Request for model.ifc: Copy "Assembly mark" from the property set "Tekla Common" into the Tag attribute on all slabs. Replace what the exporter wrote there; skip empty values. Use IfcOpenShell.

First a look at what the model holds.

```python
import ifcopenshell
import ifcopenshell.util.element

model = ifcopenshell.open("model.ifc")
print(model.schema)
slabs = model.by_type("IfcSlab")
print(len(slabs), "slabs")
for e in slabs[:8]:
    source = ifcopenshell.util.element.get_pset(e, "Tekla Common", "Assembly mark")
    target = e.Tag
    print(e.id(), repr(source), repr(target), sep=" | ")
```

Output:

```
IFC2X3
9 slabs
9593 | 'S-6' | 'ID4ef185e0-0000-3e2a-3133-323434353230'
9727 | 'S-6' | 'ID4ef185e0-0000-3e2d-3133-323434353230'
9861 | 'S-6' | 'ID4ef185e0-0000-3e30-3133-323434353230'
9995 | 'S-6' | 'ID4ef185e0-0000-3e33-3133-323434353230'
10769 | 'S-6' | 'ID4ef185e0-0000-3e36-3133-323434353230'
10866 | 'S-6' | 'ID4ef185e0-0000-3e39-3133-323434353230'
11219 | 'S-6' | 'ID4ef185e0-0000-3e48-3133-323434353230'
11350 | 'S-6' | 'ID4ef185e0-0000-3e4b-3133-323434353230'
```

```python
import ifcopenshell
import ifcopenshell.util.element

model = ifcopenshell.open("model.ifc")

count = 0
for e in model.by_type("IfcSlab"):
    value = ifcopenshell.util.element.get_pset(e, "Tekla Common", "Assembly mark")
    current = e.Tag
    if not value or not value.strip() or current == value:
        continue
    e.Tag = value
    count += 1

print(count, "slabs updated")

model.write("model_updated.ifc")
```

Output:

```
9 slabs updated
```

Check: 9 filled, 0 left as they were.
